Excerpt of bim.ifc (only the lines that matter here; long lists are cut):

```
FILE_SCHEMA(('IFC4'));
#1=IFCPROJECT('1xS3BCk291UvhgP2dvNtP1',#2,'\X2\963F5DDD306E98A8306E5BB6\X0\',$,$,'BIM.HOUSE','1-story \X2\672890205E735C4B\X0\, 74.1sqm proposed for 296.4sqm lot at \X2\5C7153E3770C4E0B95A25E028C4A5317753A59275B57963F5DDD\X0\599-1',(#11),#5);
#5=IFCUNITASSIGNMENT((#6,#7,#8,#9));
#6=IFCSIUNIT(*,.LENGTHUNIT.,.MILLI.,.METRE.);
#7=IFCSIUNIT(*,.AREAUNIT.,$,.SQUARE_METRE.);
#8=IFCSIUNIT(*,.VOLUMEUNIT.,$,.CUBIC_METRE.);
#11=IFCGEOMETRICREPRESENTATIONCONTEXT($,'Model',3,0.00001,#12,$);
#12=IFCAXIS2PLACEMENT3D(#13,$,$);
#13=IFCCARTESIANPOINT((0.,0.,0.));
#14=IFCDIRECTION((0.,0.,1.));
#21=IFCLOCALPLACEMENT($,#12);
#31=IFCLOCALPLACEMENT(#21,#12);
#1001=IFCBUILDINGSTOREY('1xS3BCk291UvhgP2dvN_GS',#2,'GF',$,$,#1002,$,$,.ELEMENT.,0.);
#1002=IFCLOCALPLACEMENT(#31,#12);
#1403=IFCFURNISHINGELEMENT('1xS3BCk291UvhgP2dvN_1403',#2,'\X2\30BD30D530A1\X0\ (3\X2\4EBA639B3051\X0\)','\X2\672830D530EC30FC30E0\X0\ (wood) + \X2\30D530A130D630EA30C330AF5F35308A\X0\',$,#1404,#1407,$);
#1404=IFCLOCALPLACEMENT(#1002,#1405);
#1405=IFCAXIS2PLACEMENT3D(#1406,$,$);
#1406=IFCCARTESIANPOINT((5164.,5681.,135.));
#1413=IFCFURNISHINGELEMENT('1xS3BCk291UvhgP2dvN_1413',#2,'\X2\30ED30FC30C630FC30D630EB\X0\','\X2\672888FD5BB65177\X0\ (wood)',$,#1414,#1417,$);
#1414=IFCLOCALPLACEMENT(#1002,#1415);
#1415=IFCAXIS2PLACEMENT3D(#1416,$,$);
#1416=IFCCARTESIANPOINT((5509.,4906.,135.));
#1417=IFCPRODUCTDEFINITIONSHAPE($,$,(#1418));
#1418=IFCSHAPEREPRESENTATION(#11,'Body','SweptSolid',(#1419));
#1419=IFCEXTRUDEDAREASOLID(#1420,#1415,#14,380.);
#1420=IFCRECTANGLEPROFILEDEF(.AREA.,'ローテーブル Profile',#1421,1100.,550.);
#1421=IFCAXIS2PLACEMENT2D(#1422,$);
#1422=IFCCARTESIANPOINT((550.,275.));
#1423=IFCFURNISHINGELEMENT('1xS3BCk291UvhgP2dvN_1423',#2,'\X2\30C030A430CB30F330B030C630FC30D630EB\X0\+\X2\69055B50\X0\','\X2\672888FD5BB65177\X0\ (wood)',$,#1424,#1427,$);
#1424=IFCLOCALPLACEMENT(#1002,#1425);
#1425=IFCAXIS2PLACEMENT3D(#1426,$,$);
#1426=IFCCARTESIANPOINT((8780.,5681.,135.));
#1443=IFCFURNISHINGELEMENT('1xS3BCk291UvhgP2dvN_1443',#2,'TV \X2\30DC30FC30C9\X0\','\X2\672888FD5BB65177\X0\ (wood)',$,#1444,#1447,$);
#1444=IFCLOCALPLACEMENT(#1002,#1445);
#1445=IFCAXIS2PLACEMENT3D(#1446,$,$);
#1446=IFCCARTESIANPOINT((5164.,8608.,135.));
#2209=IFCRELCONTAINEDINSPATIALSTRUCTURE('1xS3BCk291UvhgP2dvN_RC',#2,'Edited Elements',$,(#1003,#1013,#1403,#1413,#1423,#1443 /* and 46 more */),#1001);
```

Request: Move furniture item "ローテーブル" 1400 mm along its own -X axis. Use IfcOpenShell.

```python
import ifcopenshell
import ifcopenshell.api.geometry
import ifcopenshell.util.placement
import ifcopenshell.util.unit

model = ifcopenshell.open("bim.ifc")
unit_scale = ifcopenshell.util.unit.calculate_unit_scale(model)

item = model.by_guid("1xS3BCk291UvhgP2dvN_1413")
matrix = ifcopenshell.util.placement.get_local_placement(item.ObjectPlacement)
matrix[:3, 3] -= matrix[:3, 0] * 1.4 / unit_scale
ifcopenshell.api.geometry.edit_object_placement(model, product=item, matrix=matrix, is_si=False)

print(ifcopenshell.util.placement.get_local_placement(item.ObjectPlacement).round(3) + 0.0)

model.write("bim_v2.ifc")
```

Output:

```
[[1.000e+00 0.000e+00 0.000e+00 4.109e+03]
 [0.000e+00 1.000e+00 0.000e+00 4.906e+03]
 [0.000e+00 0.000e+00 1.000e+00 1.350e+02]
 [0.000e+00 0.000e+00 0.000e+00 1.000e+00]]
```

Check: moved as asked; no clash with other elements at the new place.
